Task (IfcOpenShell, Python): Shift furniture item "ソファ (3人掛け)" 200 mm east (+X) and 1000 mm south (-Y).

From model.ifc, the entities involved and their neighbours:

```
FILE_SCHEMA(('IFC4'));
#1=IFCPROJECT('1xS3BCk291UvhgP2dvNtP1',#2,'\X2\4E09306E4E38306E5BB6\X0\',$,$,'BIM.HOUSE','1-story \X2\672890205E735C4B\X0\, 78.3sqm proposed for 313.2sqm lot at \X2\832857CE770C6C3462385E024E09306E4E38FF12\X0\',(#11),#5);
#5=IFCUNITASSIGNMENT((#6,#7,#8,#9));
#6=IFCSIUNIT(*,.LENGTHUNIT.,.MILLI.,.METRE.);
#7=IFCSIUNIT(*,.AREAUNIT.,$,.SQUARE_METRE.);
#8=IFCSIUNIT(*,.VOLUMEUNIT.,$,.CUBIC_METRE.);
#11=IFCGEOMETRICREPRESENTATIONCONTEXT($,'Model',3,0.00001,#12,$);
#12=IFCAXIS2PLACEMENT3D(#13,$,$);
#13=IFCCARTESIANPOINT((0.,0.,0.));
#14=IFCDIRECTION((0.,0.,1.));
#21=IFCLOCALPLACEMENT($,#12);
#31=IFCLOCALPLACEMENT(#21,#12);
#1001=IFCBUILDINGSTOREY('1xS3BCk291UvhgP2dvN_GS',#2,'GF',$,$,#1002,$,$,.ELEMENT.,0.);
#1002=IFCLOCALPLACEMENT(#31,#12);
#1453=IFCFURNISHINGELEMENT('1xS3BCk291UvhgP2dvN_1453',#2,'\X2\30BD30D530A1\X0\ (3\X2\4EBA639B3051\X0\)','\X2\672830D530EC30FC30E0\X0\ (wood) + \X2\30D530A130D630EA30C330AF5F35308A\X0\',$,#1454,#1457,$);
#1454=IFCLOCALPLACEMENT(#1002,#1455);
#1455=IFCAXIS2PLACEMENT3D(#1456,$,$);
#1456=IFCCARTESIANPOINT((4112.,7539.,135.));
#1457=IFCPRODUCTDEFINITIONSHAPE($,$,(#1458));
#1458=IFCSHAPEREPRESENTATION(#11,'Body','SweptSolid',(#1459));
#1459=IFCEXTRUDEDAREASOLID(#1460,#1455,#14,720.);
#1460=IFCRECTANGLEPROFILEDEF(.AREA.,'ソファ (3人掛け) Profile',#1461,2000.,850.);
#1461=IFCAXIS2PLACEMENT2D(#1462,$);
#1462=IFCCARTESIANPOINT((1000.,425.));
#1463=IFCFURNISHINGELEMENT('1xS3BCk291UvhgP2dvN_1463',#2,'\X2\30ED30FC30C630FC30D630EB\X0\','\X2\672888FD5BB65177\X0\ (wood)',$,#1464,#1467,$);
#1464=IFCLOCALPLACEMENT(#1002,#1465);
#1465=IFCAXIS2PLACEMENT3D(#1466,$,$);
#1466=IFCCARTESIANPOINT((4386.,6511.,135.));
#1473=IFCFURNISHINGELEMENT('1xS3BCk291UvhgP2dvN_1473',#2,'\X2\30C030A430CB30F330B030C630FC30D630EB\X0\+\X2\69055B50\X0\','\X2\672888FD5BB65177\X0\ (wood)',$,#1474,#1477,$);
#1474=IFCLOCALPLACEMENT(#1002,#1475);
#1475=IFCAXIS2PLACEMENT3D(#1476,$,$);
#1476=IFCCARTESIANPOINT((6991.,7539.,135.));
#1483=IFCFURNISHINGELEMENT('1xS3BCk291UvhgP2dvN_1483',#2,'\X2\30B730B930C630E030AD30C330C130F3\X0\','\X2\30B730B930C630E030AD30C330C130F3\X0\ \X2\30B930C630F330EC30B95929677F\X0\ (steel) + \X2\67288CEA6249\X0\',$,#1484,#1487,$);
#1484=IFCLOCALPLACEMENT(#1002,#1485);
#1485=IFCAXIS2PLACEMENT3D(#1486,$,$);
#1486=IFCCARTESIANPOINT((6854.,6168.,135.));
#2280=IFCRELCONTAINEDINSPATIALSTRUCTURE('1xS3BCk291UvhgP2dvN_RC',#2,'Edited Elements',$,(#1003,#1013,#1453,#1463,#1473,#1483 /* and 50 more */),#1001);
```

```python
import ifcopenshell
import ifcopenshell.api.geometry
import ifcopenshell.util.placement
import ifcopenshell.util.unit

model = ifcopenshell.open("model.ifc")
unit_scale = ifcopenshell.util.unit.calculate_unit_scale(model)

item = model.by_guid("1xS3BCk291UvhgP2dvN_1453")
matrix = ifcopenshell.util.placement.get_local_placement(item.ObjectPlacement)
matrix[0, 3] += 0.2 / unit_scale
matrix[1, 3] -= 1 / unit_scale
ifcopenshell.api.geometry.edit_object_placement(model, product=item, matrix=matrix, is_si=False)

print(ifcopenshell.util.placement.get_local_placement(item.ObjectPlacement).round(3) + 0.0)

model.write("model_edited.ifc")
```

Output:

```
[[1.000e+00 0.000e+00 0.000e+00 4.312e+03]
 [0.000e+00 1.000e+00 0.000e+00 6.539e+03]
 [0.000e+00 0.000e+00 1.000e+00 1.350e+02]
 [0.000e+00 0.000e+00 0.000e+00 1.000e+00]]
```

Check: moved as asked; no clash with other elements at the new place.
